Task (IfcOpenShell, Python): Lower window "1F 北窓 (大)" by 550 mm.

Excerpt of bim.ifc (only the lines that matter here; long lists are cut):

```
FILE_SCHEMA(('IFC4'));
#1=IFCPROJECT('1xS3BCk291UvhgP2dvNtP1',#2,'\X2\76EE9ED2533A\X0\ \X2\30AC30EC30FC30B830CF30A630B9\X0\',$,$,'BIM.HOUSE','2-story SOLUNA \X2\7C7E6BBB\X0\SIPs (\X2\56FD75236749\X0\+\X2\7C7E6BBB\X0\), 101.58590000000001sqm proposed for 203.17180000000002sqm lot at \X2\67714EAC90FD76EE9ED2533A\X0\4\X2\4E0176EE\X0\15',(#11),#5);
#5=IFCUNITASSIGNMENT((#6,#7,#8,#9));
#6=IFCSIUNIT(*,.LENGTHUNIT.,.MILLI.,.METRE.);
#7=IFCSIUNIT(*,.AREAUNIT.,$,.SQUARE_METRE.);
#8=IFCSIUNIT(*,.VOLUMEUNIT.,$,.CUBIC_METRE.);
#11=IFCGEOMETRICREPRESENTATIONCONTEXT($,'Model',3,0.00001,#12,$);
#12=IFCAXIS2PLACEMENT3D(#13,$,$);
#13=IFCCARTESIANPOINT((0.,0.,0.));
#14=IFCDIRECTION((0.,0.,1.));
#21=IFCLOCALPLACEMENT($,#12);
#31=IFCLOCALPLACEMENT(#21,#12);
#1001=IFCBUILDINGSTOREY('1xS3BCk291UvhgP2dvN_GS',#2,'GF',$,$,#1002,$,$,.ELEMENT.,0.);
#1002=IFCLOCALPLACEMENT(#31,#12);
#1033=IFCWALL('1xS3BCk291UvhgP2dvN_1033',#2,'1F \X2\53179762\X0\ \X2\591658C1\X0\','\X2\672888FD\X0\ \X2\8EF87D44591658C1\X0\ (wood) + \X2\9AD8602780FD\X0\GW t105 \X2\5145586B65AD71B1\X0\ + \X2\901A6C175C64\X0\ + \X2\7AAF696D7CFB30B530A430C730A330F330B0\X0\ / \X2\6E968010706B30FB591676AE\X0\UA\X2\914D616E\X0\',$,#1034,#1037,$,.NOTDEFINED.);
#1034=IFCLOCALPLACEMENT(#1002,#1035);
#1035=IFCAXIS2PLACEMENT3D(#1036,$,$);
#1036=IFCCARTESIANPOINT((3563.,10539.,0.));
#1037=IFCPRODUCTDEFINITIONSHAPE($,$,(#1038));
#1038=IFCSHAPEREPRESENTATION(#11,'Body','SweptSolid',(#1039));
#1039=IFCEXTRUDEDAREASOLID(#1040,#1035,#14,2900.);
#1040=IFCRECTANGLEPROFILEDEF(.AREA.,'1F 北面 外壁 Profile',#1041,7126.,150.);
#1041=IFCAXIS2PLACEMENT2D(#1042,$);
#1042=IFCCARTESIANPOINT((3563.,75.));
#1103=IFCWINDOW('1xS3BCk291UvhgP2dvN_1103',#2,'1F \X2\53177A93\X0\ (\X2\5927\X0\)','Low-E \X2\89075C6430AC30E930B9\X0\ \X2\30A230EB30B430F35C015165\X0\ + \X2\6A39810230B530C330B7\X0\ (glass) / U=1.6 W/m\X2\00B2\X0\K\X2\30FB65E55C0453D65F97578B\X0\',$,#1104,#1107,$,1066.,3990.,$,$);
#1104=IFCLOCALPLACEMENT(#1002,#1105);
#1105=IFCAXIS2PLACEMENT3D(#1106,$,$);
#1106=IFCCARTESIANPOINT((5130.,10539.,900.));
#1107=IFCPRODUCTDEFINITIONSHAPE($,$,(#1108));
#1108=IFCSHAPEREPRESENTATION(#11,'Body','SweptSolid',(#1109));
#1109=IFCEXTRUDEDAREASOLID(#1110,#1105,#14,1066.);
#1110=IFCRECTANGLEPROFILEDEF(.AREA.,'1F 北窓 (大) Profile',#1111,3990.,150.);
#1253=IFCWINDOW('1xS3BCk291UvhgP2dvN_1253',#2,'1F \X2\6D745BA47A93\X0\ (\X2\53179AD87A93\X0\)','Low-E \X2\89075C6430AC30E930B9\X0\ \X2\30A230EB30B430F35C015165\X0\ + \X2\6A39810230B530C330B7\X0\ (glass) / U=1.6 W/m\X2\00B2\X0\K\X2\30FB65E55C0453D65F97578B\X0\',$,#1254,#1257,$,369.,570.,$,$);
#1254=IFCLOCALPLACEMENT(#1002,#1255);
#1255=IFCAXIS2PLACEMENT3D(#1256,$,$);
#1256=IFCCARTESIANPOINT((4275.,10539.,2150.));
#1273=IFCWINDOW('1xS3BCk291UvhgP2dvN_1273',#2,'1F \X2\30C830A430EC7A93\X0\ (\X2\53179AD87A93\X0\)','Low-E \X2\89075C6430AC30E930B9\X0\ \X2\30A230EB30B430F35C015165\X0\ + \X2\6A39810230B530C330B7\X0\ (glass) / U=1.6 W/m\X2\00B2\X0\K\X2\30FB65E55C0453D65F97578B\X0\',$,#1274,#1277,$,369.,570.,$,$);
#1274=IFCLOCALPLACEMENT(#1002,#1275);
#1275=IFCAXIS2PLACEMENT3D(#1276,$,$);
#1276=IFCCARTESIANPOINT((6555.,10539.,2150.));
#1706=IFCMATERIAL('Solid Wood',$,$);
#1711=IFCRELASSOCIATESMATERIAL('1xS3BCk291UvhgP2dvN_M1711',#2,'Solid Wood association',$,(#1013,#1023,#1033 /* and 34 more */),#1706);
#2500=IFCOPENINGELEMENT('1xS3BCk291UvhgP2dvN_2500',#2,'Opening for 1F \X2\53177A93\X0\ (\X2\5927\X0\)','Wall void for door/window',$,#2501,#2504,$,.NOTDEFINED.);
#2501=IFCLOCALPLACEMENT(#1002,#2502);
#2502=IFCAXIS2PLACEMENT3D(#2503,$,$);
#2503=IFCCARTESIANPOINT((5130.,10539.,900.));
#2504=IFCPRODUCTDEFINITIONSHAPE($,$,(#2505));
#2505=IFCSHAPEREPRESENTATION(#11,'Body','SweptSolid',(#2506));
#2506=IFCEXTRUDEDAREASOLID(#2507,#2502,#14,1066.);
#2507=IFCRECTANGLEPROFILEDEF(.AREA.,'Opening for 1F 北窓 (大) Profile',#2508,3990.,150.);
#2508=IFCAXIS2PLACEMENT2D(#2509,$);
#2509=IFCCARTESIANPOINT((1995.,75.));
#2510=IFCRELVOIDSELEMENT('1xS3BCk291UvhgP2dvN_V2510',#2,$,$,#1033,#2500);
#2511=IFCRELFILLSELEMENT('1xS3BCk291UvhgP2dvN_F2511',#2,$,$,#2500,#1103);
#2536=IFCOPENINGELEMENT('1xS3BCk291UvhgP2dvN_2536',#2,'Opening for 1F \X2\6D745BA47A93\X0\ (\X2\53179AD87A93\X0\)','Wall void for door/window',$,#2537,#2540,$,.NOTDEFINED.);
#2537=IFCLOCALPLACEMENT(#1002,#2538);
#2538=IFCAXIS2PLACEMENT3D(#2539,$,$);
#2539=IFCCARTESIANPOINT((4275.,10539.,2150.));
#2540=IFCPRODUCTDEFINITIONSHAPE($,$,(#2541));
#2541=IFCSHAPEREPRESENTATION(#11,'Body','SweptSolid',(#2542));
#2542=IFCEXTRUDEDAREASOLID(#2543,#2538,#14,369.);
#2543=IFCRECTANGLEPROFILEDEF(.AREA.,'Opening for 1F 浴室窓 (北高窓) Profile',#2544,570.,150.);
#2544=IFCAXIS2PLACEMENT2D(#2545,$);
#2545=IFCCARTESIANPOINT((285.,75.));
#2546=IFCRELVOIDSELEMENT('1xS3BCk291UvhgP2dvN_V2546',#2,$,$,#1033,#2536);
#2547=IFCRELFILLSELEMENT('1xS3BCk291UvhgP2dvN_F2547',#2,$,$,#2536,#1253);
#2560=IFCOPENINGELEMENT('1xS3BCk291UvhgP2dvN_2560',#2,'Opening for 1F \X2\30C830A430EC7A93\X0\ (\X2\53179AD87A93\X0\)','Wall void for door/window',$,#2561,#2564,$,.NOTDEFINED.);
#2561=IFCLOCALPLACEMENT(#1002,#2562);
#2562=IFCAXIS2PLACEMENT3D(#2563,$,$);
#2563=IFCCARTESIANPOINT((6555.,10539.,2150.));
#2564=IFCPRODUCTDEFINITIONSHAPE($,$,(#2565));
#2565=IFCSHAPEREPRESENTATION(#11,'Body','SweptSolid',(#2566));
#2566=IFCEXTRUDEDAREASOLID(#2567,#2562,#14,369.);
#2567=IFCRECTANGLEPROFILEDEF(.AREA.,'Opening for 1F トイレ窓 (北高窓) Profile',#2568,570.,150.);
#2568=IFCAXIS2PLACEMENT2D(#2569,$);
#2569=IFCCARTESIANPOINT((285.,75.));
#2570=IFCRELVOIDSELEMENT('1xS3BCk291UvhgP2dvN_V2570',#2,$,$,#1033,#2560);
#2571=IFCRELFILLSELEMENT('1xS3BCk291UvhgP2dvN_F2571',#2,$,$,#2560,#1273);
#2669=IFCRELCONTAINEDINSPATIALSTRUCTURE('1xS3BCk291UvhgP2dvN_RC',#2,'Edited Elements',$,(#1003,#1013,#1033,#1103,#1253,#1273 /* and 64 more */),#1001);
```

```python
import numpy as np
import ifcopenshell
import ifcopenshell.api.geometry
import ifcopenshell.util.placement
import ifcopenshell.util.unit

model = ifcopenshell.open("bim.ifc")
unit_scale = ifcopenshell.util.unit.calculate_unit_scale(model)

window = model.by_id(1103)
opening = window.FillsVoids[0].RelatingOpeningElement
dz = -550.0

shift = np.array([0.0, 0.0, dz])
# The window is not placed relative to its opening, so move both.
for product in (opening, window):
    matrix = ifcopenshell.util.placement.get_local_placement(product.ObjectPlacement)
    matrix[:3, 3] += shift
    ifcopenshell.api.geometry.edit_object_placement(model, product=product, matrix=matrix, is_si=False)

print(f"moved by {dz * unit_scale:+.3f} m")

model.write("bim_updated.ifc")
```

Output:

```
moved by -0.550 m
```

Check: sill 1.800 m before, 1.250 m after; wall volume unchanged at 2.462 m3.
